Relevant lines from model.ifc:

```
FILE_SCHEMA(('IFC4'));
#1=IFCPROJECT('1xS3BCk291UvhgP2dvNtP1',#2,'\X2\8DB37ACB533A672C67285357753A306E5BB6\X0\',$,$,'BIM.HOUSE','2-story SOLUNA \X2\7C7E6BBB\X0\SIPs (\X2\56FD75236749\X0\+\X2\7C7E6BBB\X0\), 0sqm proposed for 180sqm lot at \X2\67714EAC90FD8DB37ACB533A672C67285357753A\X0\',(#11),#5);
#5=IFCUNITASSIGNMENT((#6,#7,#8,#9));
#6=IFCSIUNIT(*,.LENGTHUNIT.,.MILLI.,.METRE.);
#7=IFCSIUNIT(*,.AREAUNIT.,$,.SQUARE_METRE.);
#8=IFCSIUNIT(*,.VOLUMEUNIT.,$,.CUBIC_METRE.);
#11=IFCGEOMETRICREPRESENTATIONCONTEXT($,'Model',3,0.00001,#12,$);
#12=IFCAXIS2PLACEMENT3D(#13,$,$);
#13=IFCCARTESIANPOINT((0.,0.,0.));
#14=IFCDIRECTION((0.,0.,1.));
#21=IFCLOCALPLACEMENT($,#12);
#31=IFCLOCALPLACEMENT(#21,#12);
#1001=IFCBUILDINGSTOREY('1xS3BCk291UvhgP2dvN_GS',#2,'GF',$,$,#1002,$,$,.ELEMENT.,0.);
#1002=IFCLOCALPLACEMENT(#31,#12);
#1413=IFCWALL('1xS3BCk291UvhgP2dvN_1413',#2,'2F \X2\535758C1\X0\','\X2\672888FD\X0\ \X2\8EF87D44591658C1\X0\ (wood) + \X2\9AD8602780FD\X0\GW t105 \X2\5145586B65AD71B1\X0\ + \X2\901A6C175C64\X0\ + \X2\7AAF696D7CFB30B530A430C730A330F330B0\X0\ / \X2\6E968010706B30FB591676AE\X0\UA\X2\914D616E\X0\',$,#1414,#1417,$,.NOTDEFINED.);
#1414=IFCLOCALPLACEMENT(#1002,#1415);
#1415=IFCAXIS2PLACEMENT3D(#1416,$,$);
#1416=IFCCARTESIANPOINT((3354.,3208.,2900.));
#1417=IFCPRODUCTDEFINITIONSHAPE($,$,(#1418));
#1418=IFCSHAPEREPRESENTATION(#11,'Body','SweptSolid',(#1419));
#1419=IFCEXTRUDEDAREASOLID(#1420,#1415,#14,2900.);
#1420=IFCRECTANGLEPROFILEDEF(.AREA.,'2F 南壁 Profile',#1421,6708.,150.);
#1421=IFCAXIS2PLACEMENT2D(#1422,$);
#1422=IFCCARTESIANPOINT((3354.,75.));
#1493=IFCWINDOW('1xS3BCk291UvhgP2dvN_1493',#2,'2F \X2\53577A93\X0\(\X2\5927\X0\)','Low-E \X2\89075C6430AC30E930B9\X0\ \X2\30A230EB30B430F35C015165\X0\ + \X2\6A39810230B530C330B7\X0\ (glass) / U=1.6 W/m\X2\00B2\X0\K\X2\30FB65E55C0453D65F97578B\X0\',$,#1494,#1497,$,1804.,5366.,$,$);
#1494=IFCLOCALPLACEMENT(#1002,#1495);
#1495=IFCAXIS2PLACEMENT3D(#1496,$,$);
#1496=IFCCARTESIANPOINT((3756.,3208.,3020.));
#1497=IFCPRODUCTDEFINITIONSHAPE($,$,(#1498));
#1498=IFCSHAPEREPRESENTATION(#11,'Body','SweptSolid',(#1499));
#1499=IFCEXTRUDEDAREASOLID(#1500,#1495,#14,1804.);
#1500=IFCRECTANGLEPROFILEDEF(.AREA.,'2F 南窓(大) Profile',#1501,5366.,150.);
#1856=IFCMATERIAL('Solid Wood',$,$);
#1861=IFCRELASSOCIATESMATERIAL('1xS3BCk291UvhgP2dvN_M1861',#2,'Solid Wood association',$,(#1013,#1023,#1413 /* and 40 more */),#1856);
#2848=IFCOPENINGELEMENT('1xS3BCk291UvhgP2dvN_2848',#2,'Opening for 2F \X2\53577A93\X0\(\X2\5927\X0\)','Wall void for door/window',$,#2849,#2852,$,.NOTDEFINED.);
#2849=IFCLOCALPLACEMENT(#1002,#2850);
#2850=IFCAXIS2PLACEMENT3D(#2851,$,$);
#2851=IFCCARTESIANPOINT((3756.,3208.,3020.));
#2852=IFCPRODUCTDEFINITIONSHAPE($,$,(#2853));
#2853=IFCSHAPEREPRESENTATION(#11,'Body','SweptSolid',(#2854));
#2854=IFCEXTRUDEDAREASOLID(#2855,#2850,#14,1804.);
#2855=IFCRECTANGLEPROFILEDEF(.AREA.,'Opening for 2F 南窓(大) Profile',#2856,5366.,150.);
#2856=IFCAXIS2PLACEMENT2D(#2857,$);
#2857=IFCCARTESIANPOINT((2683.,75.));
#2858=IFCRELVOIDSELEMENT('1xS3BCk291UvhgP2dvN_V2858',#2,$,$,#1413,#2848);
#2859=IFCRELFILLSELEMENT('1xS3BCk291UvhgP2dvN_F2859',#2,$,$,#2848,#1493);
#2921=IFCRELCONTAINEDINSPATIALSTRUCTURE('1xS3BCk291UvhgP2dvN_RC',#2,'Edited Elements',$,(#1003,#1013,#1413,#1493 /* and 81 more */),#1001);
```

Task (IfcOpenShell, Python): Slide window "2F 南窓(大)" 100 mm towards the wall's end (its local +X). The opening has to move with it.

```python
import ifcopenshell
import ifcopenshell.api.geometry
import ifcopenshell.util.placement
import ifcopenshell.util.unit

model = ifcopenshell.open("model.ifc")
unit_scale = ifcopenshell.util.unit.calculate_unit_scale(model)

window = model.by_guid("1xS3BCk291UvhgP2dvN_1493")
opening = window.FillsVoids[0].RelatingOpeningElement
wall = opening.VoidsElements[0].RelatingBuildingElement

wall_matrix = ifcopenshell.util.placement.get_local_placement(wall.ObjectPlacement)
shift = wall_matrix[:3, 0] * 0.1 / unit_scale
before = ifcopenshell.util.placement.get_local_placement(window.ObjectPlacement)[:3, 3].copy()

# The window is not placed relative to its opening, so move both.
for product in (opening, window):
    matrix = ifcopenshell.util.placement.get_local_placement(product.ObjectPlacement)
    matrix[:3, 3] += shift
    ifcopenshell.api.geometry.edit_object_placement(model, product=product, matrix=matrix, is_si=False)

after = ifcopenshell.util.placement.get_local_placement(window.ObjectPlacement)[:3, 3]
print("window moved by", (after - before).round(3) + 0.0)

model.write("model_edited.ifc")
```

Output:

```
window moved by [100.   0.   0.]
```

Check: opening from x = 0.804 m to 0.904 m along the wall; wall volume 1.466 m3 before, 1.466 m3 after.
